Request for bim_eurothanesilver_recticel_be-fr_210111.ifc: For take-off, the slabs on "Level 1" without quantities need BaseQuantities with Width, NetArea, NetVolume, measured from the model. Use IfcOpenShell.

First a look at what the model holds.

```python
import ifcopenshell
import ifcopenshell.util.element
import ifcopenshell.util.unit

model = ifcopenshell.open("bim_eurothanesilver_recticel_be-fr_210111.ifc")
print(model.schema)
for unit_type in ("LENGTHUNIT", "AREAUNIT", "VOLUMEUNIT"):
    print(unit_type, ifcopenshell.util.unit.calculate_unit_scale(model, unit_type))
storey = next(s for s in model.by_type("IfcBuildingStorey") if s.Name == "Level 1")
slabs = [e for e in ifcopenshell.util.element.get_decomposition(storey) if e.is_a("IfcSlab")]
for e in sorted(slabs, key=lambda e: e.id()):
    print(e.id(), e.is_a(), e.Name, list(ifcopenshell.util.element.get_psets(e, qtos_only=True)), sep=" | ")
```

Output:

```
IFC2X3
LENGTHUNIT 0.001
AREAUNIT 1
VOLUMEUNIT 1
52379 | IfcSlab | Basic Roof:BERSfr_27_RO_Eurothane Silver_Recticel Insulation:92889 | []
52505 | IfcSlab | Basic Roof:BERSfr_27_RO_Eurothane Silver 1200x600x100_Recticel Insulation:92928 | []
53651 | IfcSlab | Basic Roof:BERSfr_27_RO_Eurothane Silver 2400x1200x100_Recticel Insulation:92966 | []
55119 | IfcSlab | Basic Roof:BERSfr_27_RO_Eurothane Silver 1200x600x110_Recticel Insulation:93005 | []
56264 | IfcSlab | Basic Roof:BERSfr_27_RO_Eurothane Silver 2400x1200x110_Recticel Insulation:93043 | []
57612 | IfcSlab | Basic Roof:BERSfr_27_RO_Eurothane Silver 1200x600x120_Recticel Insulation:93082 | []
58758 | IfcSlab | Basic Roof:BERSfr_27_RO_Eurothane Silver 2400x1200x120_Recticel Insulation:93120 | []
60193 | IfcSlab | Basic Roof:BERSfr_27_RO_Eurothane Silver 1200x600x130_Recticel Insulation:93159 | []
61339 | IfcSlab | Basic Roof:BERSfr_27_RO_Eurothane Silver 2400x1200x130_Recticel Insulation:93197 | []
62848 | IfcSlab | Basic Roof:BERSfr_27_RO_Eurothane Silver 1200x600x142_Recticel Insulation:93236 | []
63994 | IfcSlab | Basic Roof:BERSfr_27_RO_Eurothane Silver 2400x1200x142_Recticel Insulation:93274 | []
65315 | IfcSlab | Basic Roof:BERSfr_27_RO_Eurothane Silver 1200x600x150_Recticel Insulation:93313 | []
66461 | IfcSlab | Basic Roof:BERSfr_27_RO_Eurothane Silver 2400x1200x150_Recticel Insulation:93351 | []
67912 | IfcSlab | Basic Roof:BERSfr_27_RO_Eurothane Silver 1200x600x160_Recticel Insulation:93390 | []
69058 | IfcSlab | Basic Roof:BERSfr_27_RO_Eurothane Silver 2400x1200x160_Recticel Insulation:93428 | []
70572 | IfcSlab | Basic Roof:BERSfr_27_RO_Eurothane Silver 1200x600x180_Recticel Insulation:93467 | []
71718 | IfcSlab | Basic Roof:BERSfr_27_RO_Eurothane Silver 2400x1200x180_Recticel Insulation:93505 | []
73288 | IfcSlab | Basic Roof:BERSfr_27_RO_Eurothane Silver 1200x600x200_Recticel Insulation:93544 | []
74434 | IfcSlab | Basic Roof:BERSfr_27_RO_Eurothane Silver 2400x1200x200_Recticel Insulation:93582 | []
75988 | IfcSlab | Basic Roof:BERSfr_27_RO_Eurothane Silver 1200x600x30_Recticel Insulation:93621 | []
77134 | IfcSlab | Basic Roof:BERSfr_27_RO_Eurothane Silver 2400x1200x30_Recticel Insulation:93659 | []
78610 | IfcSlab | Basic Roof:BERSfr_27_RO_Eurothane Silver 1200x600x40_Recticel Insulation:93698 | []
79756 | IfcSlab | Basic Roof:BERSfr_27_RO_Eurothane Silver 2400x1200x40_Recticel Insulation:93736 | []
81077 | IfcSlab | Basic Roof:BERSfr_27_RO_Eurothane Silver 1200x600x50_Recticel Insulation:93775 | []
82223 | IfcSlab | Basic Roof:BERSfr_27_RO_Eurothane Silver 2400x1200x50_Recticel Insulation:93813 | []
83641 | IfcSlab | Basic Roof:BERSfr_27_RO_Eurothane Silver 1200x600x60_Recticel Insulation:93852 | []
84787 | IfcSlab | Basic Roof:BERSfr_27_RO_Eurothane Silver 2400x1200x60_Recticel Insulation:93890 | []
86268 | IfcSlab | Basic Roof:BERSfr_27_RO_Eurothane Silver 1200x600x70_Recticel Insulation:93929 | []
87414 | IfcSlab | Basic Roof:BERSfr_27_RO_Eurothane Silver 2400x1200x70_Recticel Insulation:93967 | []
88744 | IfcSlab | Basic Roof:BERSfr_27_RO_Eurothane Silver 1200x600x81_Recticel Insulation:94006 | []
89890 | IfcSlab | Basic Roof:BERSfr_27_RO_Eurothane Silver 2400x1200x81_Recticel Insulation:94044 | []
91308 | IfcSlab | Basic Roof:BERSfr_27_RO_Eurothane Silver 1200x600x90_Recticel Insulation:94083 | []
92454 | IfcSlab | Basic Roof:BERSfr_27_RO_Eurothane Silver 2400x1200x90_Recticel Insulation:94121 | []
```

```python
import ifcopenshell
import ifcopenshell.api.pset
import ifcopenshell.geom
import ifcopenshell.util.element
import ifcopenshell.util.shape
import ifcopenshell.util.unit

model = ifcopenshell.open("bim_eurothanesilver_recticel_be-fr_210111.ifc")
unit_scale = ifcopenshell.util.unit.calculate_unit_scale(model)
area_scale = ifcopenshell.util.unit.calculate_unit_scale(model, "AREAUNIT")
volume_scale = ifcopenshell.util.unit.calculate_unit_scale(model, "VOLUMEUNIT")
settings = ifcopenshell.geom.settings()

storey = next(s for s in model.by_type("IfcBuildingStorey") if s.Name == "Level 1")
slabs = [e for e in ifcopenshell.util.element.get_decomposition(storey) if e.is_a("IfcSlab")]

for e in sorted(slabs, key=lambda e: e.id()):
    if ifcopenshell.util.element.get_psets(e, qtos_only=True, should_inherit=False):
        continue
    # Geometry comes back in metres, in the element's own axes.
    shape = ifcopenshell.geom.create_shape(settings, e)
    values = {
        "Width": ifcopenshell.util.shape.get_z(shape.geometry) / unit_scale,
        "NetArea": ifcopenshell.util.shape.get_footprint_area(shape.geometry) / area_scale,
        "NetVolume": ifcopenshell.util.shape.get_volume(shape.geometry) / volume_scale,
    }
    qto = ifcopenshell.api.pset.add_qto(model, product=e, name="BaseQuantities")
    ifcopenshell.api.pset.edit_qto(model, qto=qto, properties=values)
    print(e.id(), {k: round(v, 3) for k, v in values.items()})

model.write("bim_eurothanesilver_recticel_be-fr_210111_rev.ifc")
```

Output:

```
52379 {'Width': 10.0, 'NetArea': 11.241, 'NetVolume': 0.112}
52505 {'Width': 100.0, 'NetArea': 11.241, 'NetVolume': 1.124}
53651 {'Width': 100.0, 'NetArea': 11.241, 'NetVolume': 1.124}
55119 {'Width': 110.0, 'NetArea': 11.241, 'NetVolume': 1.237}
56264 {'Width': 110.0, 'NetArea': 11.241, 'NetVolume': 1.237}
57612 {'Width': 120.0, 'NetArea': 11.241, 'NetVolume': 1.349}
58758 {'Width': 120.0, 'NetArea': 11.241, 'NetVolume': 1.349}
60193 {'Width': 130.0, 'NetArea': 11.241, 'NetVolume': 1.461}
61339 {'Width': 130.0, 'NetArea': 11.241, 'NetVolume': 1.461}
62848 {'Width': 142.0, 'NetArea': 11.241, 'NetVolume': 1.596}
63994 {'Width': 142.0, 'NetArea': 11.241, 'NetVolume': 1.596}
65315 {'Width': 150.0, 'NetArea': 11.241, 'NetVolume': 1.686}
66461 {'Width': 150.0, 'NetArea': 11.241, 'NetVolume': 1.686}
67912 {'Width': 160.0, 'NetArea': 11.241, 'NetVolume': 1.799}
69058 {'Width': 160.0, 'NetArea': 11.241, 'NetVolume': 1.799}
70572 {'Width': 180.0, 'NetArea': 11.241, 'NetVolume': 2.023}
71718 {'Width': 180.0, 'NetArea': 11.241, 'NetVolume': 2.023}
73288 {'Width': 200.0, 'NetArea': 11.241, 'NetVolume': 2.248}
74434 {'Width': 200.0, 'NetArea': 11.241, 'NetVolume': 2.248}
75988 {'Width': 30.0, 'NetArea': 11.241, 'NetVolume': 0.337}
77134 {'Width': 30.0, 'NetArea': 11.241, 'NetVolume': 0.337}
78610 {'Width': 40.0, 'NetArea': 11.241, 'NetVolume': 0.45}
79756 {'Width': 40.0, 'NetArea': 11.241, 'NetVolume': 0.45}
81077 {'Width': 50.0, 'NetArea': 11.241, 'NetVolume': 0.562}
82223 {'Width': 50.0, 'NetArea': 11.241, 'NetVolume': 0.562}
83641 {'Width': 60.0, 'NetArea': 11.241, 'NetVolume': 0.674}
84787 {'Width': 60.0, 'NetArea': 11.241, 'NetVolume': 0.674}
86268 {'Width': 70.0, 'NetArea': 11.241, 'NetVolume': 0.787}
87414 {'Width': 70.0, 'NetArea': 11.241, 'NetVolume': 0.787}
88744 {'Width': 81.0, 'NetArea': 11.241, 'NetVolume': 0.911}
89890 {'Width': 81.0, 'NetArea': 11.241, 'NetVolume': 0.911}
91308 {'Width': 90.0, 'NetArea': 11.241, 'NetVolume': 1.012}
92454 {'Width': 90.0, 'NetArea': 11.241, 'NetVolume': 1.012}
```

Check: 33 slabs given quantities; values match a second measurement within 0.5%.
